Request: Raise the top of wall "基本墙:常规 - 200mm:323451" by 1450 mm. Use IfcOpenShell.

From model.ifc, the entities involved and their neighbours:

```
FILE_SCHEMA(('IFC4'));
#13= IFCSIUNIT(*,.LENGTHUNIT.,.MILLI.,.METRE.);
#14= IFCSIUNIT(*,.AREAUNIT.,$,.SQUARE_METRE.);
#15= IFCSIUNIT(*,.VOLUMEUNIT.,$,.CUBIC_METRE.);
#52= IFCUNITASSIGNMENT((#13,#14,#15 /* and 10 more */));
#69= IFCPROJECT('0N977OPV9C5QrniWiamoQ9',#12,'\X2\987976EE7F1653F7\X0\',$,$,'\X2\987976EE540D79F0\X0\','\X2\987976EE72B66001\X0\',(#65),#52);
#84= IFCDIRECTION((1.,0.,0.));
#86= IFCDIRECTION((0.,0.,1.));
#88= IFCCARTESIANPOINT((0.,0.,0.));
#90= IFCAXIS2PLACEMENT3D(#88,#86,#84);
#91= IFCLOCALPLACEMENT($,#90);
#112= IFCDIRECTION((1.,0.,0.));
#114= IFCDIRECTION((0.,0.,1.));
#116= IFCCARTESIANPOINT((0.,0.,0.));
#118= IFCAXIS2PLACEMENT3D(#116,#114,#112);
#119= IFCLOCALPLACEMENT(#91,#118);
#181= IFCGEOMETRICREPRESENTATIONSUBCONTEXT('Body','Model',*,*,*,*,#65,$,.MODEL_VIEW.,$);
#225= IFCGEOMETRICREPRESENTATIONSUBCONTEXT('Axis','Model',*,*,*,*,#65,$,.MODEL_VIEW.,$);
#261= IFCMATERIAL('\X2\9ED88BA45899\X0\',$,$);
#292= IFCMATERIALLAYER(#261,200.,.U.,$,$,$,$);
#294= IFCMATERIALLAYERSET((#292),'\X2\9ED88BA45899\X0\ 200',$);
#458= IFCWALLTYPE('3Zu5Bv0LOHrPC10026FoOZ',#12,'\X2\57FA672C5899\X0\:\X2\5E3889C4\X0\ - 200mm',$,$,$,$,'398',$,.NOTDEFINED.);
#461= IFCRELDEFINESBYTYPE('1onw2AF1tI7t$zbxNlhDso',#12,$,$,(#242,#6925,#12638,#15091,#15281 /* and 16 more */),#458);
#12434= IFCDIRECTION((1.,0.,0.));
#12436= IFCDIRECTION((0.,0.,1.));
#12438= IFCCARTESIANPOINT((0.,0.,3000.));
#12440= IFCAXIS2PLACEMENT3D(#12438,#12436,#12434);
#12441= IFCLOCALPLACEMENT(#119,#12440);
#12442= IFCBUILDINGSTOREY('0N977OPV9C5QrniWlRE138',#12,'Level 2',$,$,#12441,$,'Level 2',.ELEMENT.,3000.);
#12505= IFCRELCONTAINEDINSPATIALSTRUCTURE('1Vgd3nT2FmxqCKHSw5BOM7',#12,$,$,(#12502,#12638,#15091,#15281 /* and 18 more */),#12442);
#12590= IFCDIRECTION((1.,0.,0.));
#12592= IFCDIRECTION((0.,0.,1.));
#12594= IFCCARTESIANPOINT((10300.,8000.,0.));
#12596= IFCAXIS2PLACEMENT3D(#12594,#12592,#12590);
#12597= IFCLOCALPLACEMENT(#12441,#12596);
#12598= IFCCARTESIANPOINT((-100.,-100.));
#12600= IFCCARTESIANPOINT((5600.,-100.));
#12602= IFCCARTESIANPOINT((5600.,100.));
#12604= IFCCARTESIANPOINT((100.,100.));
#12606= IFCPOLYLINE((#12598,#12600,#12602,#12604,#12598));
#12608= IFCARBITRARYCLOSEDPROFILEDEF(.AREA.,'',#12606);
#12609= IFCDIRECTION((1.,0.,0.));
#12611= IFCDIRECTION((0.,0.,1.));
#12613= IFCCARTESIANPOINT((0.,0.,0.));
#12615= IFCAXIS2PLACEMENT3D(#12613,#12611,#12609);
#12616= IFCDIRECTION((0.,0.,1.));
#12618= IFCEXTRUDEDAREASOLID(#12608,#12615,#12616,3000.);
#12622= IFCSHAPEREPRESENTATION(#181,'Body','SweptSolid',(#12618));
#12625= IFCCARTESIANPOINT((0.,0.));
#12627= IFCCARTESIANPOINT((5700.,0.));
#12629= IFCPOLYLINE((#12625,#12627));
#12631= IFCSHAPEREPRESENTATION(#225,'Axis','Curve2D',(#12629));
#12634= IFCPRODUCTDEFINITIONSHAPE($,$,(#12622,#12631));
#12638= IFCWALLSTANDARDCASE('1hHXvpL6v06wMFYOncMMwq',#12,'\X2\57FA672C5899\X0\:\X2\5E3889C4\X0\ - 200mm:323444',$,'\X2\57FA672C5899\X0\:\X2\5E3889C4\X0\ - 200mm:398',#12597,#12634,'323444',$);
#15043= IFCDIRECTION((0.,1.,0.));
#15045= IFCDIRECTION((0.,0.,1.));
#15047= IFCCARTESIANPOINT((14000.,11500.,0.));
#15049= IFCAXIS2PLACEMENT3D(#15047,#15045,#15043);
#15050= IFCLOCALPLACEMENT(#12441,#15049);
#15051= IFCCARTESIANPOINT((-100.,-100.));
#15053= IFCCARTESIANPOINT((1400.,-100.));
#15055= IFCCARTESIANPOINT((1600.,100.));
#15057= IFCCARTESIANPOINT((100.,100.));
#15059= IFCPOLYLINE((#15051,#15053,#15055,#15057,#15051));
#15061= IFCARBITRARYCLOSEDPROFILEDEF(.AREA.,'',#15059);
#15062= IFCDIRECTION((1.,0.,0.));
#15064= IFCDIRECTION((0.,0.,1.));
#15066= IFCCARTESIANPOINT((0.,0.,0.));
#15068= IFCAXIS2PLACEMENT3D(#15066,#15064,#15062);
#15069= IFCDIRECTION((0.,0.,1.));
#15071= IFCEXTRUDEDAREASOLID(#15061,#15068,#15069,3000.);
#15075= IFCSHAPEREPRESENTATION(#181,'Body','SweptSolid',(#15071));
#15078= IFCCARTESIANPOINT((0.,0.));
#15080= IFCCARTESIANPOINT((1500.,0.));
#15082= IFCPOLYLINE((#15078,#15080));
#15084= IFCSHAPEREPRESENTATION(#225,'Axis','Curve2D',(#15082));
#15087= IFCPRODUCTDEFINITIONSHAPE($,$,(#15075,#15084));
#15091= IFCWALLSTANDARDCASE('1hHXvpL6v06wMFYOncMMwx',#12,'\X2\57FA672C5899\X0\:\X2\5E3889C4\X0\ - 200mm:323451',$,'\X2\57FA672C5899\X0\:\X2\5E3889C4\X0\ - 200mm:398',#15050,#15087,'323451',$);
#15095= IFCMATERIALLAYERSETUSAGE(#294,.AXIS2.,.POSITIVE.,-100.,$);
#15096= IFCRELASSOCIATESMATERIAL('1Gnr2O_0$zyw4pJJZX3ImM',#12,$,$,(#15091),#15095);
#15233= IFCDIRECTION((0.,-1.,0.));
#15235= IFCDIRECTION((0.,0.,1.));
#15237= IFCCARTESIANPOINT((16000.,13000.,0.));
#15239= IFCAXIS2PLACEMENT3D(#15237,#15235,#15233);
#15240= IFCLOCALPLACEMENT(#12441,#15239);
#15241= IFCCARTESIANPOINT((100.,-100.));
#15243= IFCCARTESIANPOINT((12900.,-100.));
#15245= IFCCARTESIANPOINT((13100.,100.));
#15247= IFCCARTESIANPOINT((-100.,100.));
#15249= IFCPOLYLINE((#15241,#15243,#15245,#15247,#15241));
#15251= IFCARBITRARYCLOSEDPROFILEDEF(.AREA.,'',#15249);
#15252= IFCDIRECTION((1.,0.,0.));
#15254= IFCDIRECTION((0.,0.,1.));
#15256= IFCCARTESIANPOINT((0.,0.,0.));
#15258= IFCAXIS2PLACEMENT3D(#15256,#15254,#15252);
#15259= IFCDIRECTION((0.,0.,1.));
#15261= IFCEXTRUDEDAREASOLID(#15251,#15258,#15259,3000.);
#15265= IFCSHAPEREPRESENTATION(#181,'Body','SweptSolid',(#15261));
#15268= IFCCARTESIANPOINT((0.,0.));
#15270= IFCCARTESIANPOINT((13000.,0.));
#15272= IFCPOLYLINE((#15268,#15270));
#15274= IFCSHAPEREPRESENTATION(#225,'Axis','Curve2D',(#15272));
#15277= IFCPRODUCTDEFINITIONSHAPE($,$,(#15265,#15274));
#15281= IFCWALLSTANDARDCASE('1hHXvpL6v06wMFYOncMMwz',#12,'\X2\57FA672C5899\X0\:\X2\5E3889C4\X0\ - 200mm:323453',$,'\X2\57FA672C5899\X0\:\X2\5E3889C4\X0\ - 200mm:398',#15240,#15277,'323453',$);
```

```python
import ifcopenshell
import ifcopenshell.geom
import ifcopenshell.util.representation
import ifcopenshell.util.shape
import ifcopenshell.util.unit

model = ifcopenshell.open("model.ifc")
unit_scale = ifcopenshell.util.unit.calculate_unit_scale(model)
settings = ifcopenshell.geom.settings()


def volume(element):
    """Net volume in cubic metres, openings subtracted."""
    shape = ifcopenshell.geom.create_shape(settings, element)
    return ifcopenshell.util.shape.get_volume(shape.geometry)


wall = model.by_id(15091)
before = volume(wall)

body = ifcopenshell.util.representation.get_representation(wall, "Model", "Body")
solid = body.Items[0]
old_height = solid.Depth
solid.Depth += 1.45 / unit_scale
after = volume(wall)

print(f"height {old_height:g} -> {solid.Depth:g}, volume {before:.3f} -> {after:.3f} m3")

model.write("model_edited.ifc")
```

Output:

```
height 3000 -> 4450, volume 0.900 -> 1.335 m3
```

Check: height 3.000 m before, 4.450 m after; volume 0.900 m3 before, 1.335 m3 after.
